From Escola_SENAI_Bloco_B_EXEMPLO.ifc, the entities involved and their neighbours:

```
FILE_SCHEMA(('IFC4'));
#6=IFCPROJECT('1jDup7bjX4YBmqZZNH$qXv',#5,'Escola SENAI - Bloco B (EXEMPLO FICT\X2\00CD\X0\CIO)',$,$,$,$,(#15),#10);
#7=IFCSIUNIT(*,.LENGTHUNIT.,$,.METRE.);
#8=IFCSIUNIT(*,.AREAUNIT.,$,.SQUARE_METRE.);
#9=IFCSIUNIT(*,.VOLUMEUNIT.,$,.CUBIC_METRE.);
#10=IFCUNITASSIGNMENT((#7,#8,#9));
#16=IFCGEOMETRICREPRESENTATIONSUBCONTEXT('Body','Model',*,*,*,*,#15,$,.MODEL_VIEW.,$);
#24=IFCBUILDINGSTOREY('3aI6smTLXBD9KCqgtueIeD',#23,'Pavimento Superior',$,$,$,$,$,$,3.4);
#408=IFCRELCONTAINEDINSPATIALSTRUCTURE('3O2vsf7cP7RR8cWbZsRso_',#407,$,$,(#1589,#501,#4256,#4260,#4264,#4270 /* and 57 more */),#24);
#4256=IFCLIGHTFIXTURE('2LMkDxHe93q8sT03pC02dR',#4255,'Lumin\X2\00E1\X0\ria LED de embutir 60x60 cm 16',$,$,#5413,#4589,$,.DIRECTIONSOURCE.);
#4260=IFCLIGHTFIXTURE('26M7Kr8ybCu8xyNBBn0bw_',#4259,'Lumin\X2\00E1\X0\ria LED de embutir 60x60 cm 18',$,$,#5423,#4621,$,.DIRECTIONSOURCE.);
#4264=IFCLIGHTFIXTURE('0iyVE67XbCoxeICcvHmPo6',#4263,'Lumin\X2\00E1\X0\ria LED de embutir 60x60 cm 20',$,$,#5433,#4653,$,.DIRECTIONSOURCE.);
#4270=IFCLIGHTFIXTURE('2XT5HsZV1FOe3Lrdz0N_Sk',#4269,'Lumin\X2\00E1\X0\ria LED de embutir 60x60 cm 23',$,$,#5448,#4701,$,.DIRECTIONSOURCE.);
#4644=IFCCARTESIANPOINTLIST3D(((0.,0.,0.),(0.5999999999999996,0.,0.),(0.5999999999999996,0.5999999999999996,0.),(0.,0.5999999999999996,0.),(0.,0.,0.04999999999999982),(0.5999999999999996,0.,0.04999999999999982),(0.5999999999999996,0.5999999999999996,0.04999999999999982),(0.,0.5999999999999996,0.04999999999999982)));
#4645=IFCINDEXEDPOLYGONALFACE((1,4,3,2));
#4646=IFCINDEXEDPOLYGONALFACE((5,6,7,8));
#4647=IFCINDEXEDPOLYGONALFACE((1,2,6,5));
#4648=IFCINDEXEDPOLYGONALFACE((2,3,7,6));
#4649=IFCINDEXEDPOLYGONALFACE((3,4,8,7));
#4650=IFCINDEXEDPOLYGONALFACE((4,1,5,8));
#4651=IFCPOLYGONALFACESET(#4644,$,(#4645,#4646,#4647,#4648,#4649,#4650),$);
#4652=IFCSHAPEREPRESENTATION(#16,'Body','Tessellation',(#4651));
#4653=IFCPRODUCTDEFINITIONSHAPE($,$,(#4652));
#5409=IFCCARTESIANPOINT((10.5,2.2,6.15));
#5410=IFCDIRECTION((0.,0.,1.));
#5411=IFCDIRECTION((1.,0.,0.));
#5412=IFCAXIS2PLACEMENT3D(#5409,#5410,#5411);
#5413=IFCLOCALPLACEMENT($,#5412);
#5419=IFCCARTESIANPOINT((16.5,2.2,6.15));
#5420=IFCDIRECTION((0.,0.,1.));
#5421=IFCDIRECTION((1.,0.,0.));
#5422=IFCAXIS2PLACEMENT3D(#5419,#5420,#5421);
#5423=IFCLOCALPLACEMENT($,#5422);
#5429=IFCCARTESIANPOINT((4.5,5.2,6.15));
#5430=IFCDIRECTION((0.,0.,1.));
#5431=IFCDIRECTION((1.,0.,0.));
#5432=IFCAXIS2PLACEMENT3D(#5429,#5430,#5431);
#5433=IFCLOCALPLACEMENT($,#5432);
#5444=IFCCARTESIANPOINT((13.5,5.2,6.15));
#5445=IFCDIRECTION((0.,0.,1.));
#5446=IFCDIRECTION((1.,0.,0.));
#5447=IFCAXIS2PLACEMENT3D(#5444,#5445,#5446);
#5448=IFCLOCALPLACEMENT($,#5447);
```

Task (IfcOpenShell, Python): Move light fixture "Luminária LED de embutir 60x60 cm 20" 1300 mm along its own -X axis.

```python
import ifcopenshell
import ifcopenshell.api.geometry
import ifcopenshell.util.placement

model = ifcopenshell.open("Escola_SENAI_Bloco_B_EXEMPLO.ifc")

item = model.by_guid("0iyVE67XbCoxeICcvHmPo6")
matrix = ifcopenshell.util.placement.get_local_placement(item.ObjectPlacement)
matrix[:3, 3] -= matrix[:3, 0] * 1.3
ifcopenshell.api.geometry.edit_object_placement(model, product=item, matrix=matrix, is_si=False)

print(ifcopenshell.util.placement.get_local_placement(item.ObjectPlacement).round(3) + 0.0)

model.write("Escola_SENAI_Bloco_B_EXEMPLO_v2.ifc")
```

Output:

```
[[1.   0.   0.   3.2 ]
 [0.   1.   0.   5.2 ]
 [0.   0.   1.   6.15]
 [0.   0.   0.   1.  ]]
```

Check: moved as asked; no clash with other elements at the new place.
